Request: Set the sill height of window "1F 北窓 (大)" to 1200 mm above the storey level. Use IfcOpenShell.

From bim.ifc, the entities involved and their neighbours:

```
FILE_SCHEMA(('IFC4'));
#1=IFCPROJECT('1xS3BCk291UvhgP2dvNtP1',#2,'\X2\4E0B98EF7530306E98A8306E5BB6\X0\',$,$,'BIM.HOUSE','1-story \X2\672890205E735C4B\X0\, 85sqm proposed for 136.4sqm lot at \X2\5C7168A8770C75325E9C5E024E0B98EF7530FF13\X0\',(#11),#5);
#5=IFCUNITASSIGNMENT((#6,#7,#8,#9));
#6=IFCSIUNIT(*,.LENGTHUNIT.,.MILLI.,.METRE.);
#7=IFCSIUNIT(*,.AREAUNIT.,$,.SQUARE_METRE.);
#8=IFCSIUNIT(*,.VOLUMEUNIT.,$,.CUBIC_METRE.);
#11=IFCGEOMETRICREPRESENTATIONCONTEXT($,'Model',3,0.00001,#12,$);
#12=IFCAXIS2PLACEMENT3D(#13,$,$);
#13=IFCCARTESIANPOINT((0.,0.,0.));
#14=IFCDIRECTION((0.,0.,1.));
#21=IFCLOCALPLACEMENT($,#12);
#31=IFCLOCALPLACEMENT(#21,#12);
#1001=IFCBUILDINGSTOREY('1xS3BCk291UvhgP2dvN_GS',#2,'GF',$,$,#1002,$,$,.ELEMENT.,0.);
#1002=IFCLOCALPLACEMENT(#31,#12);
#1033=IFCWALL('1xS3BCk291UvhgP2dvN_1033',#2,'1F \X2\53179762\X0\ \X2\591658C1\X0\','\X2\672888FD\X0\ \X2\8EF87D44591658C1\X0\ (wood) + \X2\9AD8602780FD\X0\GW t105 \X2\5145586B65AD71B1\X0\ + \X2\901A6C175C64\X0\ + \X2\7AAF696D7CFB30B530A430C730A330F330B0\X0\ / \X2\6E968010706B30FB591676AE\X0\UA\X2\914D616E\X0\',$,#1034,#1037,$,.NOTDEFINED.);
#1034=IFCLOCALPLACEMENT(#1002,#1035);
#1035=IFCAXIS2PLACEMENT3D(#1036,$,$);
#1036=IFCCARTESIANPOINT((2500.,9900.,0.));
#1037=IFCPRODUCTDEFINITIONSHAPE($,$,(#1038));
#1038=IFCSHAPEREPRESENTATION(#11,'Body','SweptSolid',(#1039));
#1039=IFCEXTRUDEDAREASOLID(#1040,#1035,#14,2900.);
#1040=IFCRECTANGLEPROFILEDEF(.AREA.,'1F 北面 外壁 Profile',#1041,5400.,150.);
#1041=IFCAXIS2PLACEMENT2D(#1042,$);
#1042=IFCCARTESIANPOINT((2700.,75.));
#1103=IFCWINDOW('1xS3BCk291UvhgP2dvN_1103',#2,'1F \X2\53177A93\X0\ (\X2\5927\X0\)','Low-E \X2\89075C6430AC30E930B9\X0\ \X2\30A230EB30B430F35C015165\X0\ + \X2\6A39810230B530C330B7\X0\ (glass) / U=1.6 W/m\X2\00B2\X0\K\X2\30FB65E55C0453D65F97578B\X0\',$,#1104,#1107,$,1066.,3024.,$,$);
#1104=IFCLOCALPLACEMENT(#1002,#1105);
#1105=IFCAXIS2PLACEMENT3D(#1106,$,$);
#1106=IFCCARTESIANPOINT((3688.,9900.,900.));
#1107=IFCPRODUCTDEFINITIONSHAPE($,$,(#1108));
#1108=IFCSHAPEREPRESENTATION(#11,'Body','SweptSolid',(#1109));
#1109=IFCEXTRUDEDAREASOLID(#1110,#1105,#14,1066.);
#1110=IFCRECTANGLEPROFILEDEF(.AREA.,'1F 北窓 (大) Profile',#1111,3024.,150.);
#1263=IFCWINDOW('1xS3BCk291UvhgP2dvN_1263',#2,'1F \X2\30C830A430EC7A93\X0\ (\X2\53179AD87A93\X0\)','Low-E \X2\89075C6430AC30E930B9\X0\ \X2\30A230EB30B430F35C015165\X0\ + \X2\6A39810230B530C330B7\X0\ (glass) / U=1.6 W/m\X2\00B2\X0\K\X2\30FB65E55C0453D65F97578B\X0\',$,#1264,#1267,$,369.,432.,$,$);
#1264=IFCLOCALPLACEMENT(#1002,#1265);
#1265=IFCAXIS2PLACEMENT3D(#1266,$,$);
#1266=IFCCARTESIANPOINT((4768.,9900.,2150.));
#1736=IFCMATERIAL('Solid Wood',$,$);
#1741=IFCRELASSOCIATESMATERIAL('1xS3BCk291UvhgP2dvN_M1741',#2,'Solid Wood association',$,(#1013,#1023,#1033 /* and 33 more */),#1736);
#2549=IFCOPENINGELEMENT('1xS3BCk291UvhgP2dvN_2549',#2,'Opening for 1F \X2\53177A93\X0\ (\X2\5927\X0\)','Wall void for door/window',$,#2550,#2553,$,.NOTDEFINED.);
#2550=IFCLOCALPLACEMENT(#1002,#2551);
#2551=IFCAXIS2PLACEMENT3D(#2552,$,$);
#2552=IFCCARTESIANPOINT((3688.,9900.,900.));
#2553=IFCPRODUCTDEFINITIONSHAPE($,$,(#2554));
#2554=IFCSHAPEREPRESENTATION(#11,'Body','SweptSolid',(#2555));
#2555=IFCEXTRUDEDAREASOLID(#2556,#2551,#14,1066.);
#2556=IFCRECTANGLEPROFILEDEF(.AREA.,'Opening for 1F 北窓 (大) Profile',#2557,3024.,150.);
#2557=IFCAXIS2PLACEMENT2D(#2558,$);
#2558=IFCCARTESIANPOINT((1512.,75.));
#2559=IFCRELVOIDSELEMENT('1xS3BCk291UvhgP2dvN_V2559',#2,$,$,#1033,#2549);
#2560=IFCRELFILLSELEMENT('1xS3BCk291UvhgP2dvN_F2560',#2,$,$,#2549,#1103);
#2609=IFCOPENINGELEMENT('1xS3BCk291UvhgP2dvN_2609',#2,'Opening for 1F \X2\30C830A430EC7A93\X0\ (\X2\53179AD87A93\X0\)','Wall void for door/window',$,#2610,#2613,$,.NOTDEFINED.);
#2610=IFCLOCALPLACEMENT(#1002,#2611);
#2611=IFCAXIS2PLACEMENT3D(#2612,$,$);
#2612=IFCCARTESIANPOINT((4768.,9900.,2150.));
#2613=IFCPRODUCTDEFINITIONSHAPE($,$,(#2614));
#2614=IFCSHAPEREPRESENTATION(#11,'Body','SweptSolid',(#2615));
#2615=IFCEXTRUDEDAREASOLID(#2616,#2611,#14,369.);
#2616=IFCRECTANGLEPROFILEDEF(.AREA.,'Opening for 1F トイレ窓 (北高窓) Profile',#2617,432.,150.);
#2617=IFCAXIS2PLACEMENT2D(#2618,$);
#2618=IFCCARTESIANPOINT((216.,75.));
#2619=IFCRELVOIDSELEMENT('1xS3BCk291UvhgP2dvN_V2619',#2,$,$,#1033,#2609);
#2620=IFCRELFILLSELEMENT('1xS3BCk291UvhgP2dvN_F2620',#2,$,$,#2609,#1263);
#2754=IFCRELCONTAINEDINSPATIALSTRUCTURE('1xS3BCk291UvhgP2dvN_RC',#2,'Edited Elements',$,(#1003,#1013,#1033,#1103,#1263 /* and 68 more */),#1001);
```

```python
import numpy as np
import ifcopenshell
import ifcopenshell.api.geometry
import ifcopenshell.geom
import ifcopenshell.util.element
import ifcopenshell.util.placement
import ifcopenshell.util.shape
import ifcopenshell.util.unit

model = ifcopenshell.open("bim.ifc")
unit_scale = ifcopenshell.util.unit.calculate_unit_scale(model)

window = model.by_id(1103)
opening = window.FillsVoids[0].RelatingOpeningElement
storey = ifcopenshell.util.element.get_container(window, ifc_class="IfcBuildingStorey")
level = ifcopenshell.util.placement.get_local_placement(storey.ObjectPlacement)[2, 3]

# The opening's origin need not be at the sill, so measure its lowest point.
shape = ifcopenshell.geom.create_shape(ifcopenshell.geom.settings(), opening)
bottom = ifcopenshell.util.shape.get_shape_bottom_elevation(shape, shape.geometry) / unit_scale
dz = level + 1.2 / unit_scale - bottom

shift = np.array([0.0, 0.0, dz])
# The window is not placed relative to its opening, so move both.
for product in (opening, window):
    matrix = ifcopenshell.util.placement.get_local_placement(product.ObjectPlacement)
    matrix[:3, 3] += shift
    ifcopenshell.api.geometry.edit_object_placement(model, product=product, matrix=matrix, is_si=False)

print(f"moved by {dz * unit_scale:+.3f} m")

model.write("bim_rev.ifc")
```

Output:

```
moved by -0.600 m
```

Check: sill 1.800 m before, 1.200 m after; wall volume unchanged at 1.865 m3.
